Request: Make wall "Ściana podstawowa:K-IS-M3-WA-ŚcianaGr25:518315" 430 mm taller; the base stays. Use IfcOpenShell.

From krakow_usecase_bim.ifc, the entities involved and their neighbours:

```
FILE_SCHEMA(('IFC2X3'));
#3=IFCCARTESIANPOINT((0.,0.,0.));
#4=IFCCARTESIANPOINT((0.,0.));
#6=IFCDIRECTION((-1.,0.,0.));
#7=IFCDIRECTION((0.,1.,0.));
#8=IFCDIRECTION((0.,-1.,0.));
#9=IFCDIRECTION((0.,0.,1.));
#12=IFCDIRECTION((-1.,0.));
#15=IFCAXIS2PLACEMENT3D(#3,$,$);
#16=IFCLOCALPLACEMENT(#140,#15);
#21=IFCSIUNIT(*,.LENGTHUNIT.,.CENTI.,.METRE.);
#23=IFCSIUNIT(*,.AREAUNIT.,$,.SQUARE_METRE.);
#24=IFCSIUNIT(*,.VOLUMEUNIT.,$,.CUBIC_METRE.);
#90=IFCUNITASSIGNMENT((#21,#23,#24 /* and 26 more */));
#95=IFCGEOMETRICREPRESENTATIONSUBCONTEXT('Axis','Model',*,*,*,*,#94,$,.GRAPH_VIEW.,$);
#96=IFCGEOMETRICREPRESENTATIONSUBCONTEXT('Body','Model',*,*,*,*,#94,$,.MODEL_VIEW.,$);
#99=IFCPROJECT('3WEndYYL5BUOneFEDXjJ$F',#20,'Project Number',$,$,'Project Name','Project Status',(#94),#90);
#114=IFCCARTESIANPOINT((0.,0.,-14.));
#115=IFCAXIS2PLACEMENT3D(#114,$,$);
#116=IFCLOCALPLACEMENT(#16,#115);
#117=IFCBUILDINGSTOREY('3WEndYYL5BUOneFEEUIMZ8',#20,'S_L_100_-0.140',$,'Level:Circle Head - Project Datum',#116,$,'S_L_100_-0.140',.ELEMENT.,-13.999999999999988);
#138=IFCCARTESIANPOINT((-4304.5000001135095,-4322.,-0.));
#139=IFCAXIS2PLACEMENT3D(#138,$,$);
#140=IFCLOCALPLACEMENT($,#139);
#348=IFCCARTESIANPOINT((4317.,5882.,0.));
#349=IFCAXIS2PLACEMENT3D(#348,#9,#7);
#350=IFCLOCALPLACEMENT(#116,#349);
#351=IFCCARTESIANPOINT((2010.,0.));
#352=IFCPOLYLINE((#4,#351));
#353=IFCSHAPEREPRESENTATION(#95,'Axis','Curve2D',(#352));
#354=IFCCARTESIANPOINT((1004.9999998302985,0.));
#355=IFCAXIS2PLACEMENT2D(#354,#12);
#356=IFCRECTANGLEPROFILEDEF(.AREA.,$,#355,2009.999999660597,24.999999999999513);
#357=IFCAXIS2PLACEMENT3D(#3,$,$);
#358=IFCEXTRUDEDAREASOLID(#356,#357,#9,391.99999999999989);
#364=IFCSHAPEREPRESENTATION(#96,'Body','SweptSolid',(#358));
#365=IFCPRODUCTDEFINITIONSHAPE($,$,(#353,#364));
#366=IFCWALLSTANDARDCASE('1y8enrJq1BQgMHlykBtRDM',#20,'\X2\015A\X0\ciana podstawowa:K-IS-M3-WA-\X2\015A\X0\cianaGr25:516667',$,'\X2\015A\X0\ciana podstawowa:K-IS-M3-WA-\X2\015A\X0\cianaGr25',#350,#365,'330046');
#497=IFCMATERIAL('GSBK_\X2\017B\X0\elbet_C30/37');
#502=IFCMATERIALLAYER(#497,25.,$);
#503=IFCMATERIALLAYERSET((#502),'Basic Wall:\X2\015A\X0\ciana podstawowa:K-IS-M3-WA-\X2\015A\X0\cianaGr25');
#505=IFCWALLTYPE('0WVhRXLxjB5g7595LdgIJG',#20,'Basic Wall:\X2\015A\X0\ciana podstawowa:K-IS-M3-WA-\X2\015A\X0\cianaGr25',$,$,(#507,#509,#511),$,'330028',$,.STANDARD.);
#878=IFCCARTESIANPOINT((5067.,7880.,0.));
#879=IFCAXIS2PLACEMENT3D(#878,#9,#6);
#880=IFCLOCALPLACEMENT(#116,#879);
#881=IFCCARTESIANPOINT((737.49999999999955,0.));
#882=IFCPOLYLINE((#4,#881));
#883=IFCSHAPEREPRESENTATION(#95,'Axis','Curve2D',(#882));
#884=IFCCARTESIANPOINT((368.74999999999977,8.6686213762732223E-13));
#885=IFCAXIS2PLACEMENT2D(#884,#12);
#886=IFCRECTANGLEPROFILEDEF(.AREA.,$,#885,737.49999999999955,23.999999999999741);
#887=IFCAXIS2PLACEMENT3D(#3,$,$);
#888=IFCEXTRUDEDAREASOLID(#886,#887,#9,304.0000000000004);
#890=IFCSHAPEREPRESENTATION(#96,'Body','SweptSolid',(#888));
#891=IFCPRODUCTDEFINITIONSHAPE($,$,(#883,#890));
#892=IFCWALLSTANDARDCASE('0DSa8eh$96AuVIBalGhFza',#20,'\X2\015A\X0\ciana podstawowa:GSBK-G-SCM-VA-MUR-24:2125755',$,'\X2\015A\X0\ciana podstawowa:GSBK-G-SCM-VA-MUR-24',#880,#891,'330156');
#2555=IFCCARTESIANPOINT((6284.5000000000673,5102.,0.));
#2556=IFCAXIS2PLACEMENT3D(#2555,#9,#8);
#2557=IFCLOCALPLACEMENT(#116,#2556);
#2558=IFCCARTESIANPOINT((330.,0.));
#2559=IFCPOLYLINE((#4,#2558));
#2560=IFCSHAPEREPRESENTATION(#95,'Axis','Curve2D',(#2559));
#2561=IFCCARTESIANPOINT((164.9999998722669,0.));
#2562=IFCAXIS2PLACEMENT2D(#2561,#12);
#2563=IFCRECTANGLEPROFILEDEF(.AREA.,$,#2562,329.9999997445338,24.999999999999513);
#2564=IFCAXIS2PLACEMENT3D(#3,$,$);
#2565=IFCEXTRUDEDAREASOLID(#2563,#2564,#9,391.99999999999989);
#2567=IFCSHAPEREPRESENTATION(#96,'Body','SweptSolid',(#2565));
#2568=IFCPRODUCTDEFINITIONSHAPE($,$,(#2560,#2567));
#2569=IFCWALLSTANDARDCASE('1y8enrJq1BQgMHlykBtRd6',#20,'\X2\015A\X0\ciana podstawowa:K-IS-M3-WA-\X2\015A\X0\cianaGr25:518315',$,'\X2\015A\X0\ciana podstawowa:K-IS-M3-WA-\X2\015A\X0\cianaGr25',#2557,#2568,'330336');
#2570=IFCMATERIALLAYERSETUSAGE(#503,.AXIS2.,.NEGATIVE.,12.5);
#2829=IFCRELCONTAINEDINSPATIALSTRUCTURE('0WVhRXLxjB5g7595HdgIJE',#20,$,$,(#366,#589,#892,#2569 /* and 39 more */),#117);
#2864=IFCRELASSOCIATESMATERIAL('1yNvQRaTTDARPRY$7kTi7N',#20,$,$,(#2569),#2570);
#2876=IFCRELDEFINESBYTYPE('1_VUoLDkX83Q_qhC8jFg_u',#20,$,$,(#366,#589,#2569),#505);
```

```python
import ifcopenshell
import ifcopenshell.geom
import ifcopenshell.util.representation
import ifcopenshell.util.shape
import ifcopenshell.util.unit

model = ifcopenshell.open("krakow_usecase_bim.ifc")
unit_scale = ifcopenshell.util.unit.calculate_unit_scale(model)
settings = ifcopenshell.geom.settings()


def volume(element):
    """Net volume in cubic metres, openings subtracted."""
    shape = ifcopenshell.geom.create_shape(settings, element)
    return ifcopenshell.util.shape.get_volume(shape.geometry)


wall = model.by_guid("1y8enrJq1BQgMHlykBtRd6")
before = volume(wall)

body = ifcopenshell.util.representation.get_representation(wall, "Model", "Body")
solid = body.Items[0]
old_height = solid.Depth
solid.Depth += 0.43 / unit_scale
after = volume(wall)

print(f"height {old_height:g} -> {solid.Depth:g}, volume {before:.3f} -> {after:.3f} m3")

model.write("krakow_usecase_bim-out.ifc")
```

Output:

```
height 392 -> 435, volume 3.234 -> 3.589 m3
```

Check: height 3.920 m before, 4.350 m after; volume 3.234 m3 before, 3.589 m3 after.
